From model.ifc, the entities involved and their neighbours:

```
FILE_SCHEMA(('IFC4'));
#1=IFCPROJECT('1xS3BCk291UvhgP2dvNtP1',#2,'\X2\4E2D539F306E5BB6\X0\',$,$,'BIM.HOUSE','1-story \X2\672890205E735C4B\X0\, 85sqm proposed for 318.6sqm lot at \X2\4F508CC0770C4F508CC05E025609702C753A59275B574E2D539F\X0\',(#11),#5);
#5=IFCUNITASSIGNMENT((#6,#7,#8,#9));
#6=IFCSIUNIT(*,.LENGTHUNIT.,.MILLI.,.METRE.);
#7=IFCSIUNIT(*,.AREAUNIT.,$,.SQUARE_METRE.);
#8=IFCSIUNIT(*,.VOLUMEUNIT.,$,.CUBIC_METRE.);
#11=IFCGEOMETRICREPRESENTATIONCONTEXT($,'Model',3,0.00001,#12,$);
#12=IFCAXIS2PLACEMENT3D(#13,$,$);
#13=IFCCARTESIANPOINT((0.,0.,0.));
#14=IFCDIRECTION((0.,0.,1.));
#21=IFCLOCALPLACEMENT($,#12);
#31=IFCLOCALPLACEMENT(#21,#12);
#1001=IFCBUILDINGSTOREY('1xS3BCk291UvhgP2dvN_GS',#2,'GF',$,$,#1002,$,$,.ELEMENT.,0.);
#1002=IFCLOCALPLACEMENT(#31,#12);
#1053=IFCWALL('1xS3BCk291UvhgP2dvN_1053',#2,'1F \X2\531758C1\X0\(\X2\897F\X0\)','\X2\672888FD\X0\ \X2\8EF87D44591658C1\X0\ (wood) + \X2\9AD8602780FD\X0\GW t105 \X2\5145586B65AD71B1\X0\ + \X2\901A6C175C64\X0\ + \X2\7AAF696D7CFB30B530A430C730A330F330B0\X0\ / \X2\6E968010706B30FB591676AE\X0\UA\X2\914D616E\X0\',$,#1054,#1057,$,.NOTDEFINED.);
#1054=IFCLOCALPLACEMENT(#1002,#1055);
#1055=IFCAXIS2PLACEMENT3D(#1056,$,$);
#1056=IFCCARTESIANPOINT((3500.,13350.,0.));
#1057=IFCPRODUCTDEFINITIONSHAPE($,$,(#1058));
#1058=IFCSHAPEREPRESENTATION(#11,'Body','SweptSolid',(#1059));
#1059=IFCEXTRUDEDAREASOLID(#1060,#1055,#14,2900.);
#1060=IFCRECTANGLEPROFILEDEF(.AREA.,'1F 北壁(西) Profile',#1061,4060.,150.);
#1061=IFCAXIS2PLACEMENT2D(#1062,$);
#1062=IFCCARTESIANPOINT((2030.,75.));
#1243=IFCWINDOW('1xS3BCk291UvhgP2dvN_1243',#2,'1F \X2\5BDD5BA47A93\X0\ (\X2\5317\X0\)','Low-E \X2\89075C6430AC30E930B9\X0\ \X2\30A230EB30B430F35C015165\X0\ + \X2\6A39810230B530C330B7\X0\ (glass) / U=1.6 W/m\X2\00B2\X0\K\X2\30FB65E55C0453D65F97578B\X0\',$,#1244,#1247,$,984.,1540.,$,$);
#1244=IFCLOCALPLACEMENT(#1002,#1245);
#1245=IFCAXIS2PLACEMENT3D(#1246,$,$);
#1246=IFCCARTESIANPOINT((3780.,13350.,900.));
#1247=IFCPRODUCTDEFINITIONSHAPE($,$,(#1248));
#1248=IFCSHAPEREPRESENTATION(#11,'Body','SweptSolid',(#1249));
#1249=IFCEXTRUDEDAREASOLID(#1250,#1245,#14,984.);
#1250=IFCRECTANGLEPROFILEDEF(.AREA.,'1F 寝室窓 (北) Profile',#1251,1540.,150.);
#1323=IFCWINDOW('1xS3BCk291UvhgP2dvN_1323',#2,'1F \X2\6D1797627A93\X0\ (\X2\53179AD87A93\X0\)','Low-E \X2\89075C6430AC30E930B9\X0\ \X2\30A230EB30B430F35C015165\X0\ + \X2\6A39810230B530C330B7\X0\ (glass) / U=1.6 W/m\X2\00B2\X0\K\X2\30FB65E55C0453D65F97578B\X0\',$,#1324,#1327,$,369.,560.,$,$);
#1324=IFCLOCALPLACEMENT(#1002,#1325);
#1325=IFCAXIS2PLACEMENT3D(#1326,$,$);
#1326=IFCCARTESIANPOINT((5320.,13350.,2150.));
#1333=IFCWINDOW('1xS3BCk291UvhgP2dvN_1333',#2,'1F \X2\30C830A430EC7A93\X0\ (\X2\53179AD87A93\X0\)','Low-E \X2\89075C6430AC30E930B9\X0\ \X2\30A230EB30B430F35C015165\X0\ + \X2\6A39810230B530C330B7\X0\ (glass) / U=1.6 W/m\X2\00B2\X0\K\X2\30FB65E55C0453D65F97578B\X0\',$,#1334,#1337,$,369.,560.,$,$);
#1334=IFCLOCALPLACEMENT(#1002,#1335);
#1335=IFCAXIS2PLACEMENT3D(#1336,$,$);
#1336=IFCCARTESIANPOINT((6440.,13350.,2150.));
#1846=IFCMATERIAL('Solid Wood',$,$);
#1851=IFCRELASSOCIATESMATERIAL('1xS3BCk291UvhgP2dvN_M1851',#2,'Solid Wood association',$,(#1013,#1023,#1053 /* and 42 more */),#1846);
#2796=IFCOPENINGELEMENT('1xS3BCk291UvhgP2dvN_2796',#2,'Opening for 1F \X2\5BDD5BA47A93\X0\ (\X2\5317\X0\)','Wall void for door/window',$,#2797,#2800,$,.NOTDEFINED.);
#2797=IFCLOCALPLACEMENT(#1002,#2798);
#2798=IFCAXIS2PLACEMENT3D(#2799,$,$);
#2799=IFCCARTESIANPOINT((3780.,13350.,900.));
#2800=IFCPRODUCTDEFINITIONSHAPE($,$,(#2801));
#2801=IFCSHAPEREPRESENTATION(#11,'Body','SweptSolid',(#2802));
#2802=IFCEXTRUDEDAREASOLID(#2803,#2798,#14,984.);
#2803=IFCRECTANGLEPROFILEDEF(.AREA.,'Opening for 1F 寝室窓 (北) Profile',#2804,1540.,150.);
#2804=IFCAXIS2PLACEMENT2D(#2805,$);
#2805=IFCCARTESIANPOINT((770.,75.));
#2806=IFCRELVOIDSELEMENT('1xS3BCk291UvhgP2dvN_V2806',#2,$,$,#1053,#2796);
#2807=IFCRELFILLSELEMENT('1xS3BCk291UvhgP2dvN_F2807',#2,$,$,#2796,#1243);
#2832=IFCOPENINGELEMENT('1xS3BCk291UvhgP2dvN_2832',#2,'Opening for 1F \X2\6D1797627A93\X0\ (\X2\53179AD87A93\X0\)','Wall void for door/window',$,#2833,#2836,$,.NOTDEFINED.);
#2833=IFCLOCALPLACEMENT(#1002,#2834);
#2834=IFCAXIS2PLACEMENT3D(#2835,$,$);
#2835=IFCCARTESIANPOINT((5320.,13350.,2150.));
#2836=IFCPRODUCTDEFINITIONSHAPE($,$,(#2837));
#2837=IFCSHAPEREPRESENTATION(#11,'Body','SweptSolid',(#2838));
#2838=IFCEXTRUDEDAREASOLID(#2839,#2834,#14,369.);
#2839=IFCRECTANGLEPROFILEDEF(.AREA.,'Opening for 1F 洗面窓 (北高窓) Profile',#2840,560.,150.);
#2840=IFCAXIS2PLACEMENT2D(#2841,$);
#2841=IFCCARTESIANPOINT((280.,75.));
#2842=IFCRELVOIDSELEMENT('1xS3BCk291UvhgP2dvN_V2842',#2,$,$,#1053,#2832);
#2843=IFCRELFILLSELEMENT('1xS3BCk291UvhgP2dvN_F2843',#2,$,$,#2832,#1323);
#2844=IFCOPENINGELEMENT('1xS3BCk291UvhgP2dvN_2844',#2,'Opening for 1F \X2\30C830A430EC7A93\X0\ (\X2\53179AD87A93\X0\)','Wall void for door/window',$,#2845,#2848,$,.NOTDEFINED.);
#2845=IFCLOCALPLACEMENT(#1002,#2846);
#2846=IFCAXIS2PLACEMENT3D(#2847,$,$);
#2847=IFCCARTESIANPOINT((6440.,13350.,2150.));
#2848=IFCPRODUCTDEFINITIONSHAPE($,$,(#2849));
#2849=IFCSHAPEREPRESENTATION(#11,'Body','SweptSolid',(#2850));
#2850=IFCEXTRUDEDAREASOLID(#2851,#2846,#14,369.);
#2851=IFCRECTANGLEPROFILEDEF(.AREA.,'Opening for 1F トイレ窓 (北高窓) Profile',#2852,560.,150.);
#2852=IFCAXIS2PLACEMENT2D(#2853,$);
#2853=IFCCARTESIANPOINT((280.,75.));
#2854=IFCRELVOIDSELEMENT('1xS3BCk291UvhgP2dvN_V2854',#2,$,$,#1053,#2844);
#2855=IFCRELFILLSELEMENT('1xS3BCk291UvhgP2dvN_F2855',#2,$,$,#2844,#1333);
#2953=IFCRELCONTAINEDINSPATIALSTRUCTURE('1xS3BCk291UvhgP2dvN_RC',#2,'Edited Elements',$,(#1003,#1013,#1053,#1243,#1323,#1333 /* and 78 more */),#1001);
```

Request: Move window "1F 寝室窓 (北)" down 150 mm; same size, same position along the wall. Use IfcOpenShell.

```python
import numpy as np
import ifcopenshell
import ifcopenshell.api.geometry
import ifcopenshell.util.placement
import ifcopenshell.util.unit

model = ifcopenshell.open("model.ifc")
unit_scale = ifcopenshell.util.unit.calculate_unit_scale(model)

window = model.by_id(1243)
opening = window.FillsVoids[0].RelatingOpeningElement
dz = -0.15 / unit_scale

shift = np.array([0.0, 0.0, dz])
# The window is not placed relative to its opening, so move both.
for product in (opening, window):
    matrix = ifcopenshell.util.placement.get_local_placement(product.ObjectPlacement)
    matrix[:3, 3] += shift
    ifcopenshell.api.geometry.edit_object_placement(model, product=product, matrix=matrix, is_si=False)

print(f"moved by {dz * unit_scale:+.3f} m")

model.write("model-out.ifc")
```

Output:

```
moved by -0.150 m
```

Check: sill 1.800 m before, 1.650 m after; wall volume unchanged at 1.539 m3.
